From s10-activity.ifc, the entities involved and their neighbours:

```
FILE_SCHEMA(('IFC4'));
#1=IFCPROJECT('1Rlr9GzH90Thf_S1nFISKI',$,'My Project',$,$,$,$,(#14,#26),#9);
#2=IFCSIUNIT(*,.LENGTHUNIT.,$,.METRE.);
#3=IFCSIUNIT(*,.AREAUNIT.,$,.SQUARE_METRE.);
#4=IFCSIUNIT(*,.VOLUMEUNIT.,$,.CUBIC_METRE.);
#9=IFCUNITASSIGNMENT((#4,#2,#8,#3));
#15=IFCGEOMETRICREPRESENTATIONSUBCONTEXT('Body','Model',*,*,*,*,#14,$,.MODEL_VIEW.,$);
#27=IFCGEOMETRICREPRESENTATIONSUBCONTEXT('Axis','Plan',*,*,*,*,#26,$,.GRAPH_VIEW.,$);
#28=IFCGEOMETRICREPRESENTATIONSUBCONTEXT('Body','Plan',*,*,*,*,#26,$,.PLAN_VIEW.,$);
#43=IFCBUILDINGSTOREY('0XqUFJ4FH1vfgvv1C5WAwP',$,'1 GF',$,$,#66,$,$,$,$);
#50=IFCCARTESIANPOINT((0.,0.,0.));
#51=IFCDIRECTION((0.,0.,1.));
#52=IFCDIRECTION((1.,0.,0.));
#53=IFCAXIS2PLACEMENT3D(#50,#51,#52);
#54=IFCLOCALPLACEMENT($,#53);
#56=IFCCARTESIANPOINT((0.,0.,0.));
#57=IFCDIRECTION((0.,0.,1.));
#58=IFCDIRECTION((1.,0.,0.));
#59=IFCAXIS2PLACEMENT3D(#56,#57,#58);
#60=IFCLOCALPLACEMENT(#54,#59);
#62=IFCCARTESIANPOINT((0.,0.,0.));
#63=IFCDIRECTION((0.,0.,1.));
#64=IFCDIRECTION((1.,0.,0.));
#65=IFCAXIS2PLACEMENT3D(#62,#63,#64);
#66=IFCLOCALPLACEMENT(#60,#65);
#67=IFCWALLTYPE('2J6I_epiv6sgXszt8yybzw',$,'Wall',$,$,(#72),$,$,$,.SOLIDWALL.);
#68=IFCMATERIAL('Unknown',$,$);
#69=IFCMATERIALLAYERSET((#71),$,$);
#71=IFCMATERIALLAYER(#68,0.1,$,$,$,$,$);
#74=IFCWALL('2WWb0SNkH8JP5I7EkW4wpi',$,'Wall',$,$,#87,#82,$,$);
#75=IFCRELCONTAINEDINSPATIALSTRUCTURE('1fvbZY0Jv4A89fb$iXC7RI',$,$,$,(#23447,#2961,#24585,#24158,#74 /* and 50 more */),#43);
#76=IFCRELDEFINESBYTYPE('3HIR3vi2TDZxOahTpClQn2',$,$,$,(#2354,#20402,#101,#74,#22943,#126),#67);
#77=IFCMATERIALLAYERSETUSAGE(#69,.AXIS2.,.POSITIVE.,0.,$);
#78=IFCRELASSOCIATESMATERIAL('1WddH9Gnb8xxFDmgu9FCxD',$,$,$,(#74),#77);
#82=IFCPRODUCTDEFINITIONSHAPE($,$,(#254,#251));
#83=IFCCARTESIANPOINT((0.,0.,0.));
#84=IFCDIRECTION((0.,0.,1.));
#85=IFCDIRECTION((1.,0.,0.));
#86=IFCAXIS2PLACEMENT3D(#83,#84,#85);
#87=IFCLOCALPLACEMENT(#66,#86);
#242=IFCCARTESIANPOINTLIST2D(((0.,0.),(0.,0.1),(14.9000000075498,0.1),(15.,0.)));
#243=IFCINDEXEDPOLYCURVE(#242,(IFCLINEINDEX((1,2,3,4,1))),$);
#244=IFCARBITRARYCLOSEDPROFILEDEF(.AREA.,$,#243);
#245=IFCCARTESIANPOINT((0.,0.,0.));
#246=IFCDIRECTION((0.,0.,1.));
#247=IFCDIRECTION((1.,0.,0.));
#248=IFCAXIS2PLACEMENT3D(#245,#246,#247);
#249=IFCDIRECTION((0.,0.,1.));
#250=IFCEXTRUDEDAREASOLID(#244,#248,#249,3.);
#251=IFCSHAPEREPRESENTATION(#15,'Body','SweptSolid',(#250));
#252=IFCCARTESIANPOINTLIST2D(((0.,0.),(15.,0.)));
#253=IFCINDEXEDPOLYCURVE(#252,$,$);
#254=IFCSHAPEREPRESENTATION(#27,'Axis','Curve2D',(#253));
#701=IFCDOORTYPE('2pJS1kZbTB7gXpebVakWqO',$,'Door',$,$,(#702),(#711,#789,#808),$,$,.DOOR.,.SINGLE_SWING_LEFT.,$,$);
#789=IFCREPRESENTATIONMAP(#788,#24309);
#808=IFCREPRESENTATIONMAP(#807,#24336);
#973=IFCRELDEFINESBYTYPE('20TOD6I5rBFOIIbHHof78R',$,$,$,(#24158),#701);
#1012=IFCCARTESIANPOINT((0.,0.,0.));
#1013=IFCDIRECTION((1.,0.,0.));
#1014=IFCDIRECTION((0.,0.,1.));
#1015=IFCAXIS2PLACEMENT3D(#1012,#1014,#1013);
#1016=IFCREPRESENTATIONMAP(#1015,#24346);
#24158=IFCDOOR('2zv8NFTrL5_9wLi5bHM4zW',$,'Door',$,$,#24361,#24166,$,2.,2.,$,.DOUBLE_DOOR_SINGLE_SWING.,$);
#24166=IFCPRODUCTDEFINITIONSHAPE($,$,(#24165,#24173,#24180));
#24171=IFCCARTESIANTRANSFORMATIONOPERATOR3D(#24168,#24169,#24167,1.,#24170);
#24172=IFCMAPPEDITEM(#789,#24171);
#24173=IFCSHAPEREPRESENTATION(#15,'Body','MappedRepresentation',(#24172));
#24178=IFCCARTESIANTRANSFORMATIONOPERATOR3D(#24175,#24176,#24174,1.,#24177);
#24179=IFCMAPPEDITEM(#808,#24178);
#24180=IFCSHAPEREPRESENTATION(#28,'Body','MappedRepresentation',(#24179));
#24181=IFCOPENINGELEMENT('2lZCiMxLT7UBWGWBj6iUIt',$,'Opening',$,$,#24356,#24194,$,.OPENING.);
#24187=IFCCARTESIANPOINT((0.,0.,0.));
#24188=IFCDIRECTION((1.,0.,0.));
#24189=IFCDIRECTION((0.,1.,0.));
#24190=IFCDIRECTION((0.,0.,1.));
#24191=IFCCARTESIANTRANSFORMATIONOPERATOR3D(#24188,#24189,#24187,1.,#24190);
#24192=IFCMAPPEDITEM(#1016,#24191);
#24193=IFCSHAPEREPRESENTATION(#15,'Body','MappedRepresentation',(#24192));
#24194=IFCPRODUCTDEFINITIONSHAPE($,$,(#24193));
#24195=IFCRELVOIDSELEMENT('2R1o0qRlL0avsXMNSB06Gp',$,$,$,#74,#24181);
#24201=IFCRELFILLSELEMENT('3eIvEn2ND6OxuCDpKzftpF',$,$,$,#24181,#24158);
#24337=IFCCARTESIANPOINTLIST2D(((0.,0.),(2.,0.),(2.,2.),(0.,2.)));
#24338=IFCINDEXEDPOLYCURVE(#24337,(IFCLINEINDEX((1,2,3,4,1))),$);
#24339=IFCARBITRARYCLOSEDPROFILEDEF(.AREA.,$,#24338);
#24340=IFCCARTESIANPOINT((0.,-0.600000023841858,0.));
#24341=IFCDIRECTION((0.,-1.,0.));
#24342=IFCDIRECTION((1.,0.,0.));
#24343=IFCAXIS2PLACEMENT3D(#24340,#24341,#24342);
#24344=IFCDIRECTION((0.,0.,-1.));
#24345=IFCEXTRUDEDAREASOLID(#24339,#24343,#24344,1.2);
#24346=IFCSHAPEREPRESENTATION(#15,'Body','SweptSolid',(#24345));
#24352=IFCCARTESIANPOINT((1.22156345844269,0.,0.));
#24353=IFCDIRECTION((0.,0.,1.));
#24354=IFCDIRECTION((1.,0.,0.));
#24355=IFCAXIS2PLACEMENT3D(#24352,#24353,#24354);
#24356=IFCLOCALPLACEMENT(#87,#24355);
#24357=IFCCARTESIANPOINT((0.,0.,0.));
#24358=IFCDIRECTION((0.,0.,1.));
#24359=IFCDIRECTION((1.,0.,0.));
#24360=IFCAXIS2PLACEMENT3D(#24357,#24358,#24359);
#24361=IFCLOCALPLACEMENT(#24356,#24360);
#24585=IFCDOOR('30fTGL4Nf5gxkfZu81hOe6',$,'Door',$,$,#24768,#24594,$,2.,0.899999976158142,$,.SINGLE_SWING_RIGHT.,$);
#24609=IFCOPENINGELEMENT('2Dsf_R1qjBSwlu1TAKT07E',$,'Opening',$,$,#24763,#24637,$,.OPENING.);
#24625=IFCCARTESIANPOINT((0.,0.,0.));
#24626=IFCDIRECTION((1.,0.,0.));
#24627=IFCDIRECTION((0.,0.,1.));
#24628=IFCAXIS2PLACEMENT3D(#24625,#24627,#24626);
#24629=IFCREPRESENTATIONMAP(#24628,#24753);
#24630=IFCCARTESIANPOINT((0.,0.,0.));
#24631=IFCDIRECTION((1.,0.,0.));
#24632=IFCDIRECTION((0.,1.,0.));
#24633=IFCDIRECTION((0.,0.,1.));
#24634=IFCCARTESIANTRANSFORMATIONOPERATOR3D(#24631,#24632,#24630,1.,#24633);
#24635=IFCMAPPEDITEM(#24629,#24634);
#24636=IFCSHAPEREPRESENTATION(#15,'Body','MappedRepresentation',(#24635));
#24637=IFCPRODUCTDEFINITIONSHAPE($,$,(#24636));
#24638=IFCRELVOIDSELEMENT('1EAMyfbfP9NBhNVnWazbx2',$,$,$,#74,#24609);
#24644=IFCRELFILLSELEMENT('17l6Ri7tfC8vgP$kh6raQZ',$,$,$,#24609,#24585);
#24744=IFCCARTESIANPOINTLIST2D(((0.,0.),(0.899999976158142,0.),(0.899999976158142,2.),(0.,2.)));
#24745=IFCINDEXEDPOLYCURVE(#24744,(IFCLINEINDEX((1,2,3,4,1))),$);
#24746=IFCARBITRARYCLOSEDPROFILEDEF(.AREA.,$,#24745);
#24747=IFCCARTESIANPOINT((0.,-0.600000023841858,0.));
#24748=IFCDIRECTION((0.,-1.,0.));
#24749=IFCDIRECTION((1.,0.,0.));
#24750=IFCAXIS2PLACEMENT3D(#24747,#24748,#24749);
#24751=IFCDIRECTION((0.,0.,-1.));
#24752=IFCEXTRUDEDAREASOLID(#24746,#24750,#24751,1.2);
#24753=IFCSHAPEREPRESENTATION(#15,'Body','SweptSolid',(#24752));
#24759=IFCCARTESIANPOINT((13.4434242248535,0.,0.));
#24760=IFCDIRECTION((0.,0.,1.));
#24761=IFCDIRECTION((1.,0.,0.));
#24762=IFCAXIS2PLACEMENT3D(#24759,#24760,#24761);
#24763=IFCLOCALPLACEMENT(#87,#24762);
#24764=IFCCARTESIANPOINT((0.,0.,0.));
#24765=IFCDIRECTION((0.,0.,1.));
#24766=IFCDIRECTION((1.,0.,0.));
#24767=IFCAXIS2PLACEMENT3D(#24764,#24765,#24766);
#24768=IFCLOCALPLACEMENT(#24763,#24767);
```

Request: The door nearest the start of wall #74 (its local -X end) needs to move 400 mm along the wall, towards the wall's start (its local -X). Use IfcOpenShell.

```python
import ifcopenshell
import ifcopenshell.api.geometry
import ifcopenshell.util.placement

model = ifcopenshell.open("s10-activity.ifc")

door = model.by_guid("2zv8NFTrL5_9wLi5bHM4zW")
opening = door.FillsVoids[0].RelatingOpeningElement
wall = opening.VoidsElements[0].RelatingBuildingElement

wall_matrix = ifcopenshell.util.placement.get_local_placement(wall.ObjectPlacement)
shift = wall_matrix[:3, 0] * -0.4
before = ifcopenshell.util.placement.get_local_placement(door.ObjectPlacement)[:3, 3].copy()

# The door is placed relative to its opening, so it follows when the opening moves.
matrix = ifcopenshell.util.placement.get_local_placement(opening.ObjectPlacement)
matrix[:3, 3] += shift
ifcopenshell.api.geometry.edit_object_placement(
    model, product=opening, matrix=matrix, is_si=False, should_transform_children=True
)

after = ifcopenshell.util.placement.get_local_placement(door.ObjectPlacement)[:3, 3]
print("door moved by", (after - before).round(3) + 0.0)

model.write("s10-activity-out.ifc")
```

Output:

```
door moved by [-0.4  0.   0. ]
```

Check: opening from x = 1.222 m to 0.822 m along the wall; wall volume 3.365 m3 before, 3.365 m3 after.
